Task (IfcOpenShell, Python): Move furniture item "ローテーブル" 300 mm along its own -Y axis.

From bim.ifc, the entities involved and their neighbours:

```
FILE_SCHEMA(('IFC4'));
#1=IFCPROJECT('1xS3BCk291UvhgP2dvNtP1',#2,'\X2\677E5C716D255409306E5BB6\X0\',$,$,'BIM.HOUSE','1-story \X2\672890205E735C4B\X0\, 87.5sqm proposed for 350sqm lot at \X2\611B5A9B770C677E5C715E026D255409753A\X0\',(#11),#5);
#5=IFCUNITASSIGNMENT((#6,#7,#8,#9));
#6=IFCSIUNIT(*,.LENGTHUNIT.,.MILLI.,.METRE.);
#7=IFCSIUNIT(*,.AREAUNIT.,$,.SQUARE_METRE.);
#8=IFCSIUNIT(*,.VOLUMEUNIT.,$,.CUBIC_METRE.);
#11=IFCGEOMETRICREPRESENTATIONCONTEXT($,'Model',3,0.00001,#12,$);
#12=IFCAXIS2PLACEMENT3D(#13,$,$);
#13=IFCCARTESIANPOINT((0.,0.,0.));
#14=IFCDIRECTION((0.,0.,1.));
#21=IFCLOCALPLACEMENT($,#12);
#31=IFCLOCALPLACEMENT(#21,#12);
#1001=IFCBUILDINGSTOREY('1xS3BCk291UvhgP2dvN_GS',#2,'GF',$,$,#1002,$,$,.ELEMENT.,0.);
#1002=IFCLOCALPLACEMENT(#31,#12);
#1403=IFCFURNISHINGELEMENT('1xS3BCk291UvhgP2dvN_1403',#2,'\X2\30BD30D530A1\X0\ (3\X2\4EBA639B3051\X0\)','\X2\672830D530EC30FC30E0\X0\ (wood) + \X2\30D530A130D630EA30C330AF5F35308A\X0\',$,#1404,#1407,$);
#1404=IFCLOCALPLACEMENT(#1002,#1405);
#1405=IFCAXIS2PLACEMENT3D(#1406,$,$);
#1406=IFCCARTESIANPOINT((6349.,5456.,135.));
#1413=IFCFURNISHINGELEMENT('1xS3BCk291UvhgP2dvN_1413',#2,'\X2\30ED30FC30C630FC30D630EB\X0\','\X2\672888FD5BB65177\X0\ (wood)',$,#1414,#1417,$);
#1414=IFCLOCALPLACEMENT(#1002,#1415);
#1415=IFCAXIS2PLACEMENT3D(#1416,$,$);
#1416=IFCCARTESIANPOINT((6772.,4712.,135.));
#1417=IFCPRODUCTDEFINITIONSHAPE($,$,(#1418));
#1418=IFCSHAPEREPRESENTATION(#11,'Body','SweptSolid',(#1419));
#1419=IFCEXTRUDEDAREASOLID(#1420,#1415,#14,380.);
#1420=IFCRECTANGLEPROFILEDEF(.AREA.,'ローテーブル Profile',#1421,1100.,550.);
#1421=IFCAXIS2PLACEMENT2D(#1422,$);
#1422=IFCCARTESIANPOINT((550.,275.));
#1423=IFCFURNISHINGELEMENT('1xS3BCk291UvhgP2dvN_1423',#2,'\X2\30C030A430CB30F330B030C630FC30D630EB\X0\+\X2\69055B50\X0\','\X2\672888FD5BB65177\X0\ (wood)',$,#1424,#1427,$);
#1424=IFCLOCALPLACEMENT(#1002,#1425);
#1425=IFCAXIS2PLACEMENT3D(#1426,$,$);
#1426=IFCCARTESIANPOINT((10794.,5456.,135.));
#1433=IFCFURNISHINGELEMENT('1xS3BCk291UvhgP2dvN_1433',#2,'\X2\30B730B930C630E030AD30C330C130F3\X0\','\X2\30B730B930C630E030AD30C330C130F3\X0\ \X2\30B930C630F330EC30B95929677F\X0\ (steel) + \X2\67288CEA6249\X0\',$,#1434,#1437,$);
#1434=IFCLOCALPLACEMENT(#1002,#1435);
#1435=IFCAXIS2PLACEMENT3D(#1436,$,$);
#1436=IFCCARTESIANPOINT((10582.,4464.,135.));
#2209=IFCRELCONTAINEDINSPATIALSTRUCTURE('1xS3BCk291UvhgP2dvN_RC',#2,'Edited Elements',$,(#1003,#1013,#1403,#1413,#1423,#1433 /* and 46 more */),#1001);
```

```python
import ifcopenshell
import ifcopenshell.api.geometry
import ifcopenshell.util.placement
import ifcopenshell.util.unit

model = ifcopenshell.open("bim.ifc")
unit_scale = ifcopenshell.util.unit.calculate_unit_scale(model)

item = model.by_guid("1xS3BCk291UvhgP2dvN_1413")
matrix = ifcopenshell.util.placement.get_local_placement(item.ObjectPlacement)
matrix[:3, 3] -= matrix[:3, 1] * 0.3 / unit_scale
ifcopenshell.api.geometry.edit_object_placement(model, product=item, matrix=matrix, is_si=False)

print(ifcopenshell.util.placement.get_local_placement(item.ObjectPlacement).round(3) + 0.0)

model.write("bim-out.ifc")
```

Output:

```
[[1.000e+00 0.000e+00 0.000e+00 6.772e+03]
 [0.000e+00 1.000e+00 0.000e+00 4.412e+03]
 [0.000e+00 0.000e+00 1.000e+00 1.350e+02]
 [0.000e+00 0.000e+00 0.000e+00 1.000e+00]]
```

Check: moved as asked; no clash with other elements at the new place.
